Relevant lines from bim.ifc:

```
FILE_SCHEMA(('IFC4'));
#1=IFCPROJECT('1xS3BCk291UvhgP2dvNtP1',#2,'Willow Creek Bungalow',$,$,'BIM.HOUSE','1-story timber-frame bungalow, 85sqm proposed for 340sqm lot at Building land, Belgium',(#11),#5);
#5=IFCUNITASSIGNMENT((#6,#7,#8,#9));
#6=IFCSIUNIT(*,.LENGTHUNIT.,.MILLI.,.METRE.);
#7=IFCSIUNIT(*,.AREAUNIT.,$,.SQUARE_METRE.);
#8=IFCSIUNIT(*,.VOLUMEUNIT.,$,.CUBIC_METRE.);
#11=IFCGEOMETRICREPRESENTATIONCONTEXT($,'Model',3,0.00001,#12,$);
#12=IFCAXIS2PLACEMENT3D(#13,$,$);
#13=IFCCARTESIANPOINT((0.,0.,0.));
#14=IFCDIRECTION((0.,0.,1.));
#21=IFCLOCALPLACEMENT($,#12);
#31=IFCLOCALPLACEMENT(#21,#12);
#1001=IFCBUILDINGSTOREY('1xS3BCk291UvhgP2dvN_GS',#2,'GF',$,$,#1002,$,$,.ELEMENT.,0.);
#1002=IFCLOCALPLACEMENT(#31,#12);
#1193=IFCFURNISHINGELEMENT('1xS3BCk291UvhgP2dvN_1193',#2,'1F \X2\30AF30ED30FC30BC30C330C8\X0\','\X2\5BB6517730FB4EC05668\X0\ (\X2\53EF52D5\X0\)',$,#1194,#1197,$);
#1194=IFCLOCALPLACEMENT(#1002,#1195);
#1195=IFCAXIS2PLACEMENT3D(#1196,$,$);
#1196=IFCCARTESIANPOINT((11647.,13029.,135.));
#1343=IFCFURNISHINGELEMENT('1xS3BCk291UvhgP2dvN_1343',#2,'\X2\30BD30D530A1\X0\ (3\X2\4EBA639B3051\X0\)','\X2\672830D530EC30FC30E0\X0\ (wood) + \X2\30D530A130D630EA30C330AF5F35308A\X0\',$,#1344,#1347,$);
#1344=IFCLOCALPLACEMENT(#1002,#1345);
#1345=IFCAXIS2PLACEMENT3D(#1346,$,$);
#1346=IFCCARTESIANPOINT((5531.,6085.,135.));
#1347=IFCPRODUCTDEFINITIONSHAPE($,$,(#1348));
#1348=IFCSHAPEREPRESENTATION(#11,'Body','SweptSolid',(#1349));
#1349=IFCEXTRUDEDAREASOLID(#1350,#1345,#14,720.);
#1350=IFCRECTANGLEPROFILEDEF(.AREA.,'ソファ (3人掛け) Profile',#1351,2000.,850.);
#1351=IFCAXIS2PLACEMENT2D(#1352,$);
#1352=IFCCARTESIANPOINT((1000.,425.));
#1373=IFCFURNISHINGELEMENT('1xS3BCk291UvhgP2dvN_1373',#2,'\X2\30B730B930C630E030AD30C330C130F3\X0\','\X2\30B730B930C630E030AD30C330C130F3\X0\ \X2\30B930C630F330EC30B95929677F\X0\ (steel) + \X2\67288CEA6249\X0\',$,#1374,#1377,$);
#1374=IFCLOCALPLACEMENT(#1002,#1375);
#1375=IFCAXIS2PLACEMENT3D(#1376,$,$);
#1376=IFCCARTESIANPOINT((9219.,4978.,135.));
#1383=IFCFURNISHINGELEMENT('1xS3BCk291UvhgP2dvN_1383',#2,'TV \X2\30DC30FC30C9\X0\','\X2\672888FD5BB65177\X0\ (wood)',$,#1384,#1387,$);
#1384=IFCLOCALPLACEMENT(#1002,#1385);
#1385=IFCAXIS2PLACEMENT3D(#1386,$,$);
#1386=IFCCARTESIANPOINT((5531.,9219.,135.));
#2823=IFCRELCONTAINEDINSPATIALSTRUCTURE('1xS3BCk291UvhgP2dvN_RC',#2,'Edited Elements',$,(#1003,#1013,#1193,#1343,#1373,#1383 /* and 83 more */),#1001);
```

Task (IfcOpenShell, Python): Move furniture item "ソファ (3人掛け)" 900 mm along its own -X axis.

```python
import ifcopenshell
import ifcopenshell.api.geometry
import ifcopenshell.util.placement
import ifcopenshell.util.unit

model = ifcopenshell.open("bim.ifc")
unit_scale = ifcopenshell.util.unit.calculate_unit_scale(model)

item = model.by_id(1343)
matrix = ifcopenshell.util.placement.get_local_placement(item.ObjectPlacement)
matrix[:3, 3] -= matrix[:3, 0] * 0.9 / unit_scale
ifcopenshell.api.geometry.edit_object_placement(model, product=item, matrix=matrix, is_si=False)

print(ifcopenshell.util.placement.get_local_placement(item.ObjectPlacement).round(3) + 0.0)

model.write("bim_v2.ifc")
```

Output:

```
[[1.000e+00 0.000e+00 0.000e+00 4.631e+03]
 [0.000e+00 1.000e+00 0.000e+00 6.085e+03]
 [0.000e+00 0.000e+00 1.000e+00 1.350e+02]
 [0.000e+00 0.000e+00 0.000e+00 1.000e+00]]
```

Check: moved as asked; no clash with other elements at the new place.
